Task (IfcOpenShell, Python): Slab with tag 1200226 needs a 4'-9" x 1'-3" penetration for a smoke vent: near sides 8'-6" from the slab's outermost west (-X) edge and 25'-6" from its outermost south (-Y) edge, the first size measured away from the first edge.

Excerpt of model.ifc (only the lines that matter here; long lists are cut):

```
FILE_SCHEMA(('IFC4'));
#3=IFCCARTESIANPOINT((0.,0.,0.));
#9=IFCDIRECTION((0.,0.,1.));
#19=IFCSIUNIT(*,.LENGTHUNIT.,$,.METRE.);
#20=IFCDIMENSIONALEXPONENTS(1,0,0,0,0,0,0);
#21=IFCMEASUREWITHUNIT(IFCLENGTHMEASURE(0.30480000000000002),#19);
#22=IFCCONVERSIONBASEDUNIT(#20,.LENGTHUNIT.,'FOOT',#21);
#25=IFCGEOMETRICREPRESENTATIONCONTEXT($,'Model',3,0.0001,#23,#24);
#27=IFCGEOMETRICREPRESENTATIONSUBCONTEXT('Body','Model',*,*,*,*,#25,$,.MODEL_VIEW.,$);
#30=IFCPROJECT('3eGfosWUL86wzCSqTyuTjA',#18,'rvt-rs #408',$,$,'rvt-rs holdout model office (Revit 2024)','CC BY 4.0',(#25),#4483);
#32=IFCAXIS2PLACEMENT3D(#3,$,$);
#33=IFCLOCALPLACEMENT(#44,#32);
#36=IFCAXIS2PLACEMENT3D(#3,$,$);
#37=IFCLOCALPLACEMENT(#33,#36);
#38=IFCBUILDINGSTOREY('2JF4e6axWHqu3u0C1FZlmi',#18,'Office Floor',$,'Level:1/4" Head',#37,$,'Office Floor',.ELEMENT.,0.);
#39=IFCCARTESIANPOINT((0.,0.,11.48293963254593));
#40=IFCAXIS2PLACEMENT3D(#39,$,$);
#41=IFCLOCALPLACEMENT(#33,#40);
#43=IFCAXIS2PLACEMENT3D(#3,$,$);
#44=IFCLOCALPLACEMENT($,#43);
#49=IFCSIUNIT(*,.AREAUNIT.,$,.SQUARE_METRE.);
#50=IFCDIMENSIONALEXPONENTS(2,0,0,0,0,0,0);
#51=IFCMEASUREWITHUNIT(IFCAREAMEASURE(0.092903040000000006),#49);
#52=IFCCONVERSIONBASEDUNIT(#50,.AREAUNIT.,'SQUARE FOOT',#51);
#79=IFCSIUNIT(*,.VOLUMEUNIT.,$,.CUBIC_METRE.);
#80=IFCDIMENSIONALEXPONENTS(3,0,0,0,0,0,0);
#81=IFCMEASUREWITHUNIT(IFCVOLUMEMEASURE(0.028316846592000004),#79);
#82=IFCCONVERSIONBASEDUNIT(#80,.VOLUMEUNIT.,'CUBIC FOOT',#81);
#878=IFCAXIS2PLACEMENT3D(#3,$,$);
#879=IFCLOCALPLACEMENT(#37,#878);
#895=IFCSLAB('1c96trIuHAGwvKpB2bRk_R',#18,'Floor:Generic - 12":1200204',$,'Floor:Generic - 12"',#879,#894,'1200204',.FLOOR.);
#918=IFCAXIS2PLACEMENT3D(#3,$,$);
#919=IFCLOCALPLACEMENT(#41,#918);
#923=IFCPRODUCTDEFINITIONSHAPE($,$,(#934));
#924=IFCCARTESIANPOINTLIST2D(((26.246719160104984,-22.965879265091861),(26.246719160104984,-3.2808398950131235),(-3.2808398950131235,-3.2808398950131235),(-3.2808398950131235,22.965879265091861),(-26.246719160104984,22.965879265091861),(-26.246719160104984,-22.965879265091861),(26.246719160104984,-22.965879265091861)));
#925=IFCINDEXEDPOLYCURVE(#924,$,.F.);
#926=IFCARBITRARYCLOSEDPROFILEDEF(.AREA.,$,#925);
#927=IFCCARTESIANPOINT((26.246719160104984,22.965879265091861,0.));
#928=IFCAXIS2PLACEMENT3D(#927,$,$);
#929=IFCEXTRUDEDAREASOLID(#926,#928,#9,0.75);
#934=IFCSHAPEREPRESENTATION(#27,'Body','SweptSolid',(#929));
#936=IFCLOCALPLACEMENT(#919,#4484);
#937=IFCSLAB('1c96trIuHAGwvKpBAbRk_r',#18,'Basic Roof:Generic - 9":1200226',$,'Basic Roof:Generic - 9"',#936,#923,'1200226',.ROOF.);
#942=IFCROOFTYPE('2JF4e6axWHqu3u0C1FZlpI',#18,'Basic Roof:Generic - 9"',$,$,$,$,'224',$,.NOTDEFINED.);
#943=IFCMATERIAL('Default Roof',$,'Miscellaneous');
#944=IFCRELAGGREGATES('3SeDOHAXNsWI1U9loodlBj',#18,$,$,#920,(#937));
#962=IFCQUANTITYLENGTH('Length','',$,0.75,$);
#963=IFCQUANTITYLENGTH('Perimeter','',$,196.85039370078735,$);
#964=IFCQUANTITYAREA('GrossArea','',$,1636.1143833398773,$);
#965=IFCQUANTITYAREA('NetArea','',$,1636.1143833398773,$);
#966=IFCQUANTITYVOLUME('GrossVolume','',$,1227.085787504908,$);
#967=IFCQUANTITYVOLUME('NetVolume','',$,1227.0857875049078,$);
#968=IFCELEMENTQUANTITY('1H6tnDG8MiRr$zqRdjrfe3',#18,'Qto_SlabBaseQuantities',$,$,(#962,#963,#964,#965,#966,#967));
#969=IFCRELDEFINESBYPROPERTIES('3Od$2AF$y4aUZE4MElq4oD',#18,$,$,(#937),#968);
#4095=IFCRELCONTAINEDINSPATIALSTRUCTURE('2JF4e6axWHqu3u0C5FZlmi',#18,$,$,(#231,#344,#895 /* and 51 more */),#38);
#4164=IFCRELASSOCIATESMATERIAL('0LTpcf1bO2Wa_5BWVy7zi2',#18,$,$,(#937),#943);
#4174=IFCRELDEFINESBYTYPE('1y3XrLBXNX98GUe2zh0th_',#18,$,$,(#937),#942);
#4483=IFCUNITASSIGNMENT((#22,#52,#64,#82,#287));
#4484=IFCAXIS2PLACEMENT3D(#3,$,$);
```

```python
import numpy as np
import ifcopenshell
import ifcopenshell.api.feature
import ifcopenshell.api.geometry
import ifcopenshell.api.pset
import ifcopenshell.api.root
import ifcopenshell.geom
import ifcopenshell.util.element
import ifcopenshell.util.placement
import ifcopenshell.util.representation
import ifcopenshell.util.shape
import ifcopenshell.util.unit

model = ifcopenshell.open("model.ifc")
unit_scale = ifcopenshell.util.unit.calculate_unit_scale(model)
area_scale = ifcopenshell.util.unit.calculate_unit_scale(model, "AREAUNIT")
volume_scale = ifcopenshell.util.unit.calculate_unit_scale(model, "VOLUMEUNIT")
settings = ifcopenshell.geom.settings()


def volume(element):
    """Net volume in cubic metres, openings subtracted."""
    shape = ifcopenshell.geom.create_shape(settings, element)
    return ifcopenshell.util.shape.get_volume(shape.geometry)


slab = model.by_id(937)
before = volume(slab)

# Extent in the slab's own axes, in metres. The edges named are its -X and -Y sides.
slab_shape = ifcopenshell.geom.create_shape(settings, slab)
vertices = ifcopenshell.util.shape.get_vertices(slab_shape.geometry)
x_min, y_min, bottom = vertices.min(axis=0)
top = vertices[:, 2].max()

opening = ifcopenshell.api.root.create_entity(model, ifc_class="IfcOpeningElement", name="Smoke vent opening", predefined_type="OPENING")
context = ifcopenshell.util.representation.get_context(model, "Model", "Body", "MODEL_VIEW")
width, depth = 1.4478, 0.381
outline = [(0.0, 0.0), (width, 0.0), (width, depth), (0.0, depth), (0.0, 0.0)]
# Overshoot both faces by 50 mm so the cut is clean.
shape = ifcopenshell.api.geometry.add_slab_representation(
    model, context=context, depth=top - bottom + 0.1, polyline=outline
)
ifcopenshell.api.geometry.assign_representation(model, product=opening, representation=shape)

matrix = ifcopenshell.util.placement.get_local_placement(slab.ObjectPlacement)
matrix[:, 3] = matrix @ np.append(np.array([x_min + 2.5908, y_min + 7.7724, bottom - 0.05]) / unit_scale, 1.0)
ifcopenshell.api.geometry.edit_object_placement(model, product=opening, matrix=matrix, is_si=False)
ifcopenshell.api.feature.add_feature(model, feature=opening, element=slab)

after = volume(slab)

# Update the slab's stored quantities.
qto = model.by_id(ifcopenshell.util.element.get_pset(slab, "Qto_SlabBaseQuantities", should_inherit=False)["id"])
ifcopenshell.api.pset.edit_qto(model, qto=qto, properties={
    "NetArea": after / (top - bottom) / area_scale,
    "NetVolume": after / volume_scale,
})

print(f"slab volume {before:.3f} -> {after:.3f} m3")

model.write("model-out.ifc")
```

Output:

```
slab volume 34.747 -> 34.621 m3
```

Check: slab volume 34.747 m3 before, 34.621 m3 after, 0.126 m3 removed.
